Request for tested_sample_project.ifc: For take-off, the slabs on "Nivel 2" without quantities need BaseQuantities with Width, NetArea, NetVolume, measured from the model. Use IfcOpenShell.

First a look at what the model holds.

```python
import ifcopenshell
import ifcopenshell.util.element
import ifcopenshell.util.unit

model = ifcopenshell.open("tested_sample_project.ifc")
print(model.schema)
for unit_type in ("LENGTHUNIT", "AREAUNIT", "VOLUMEUNIT"):
    print(unit_type, ifcopenshell.util.unit.calculate_unit_scale(model, unit_type))
storey = next(s for s in model.by_type("IfcBuildingStorey") if s.Name == "Nivel 2")
slabs = [e for e in ifcopenshell.util.element.get_decomposition(storey) if e.is_a("IfcSlab")]
for e in sorted(slabs, key=lambda e: e.id()):
    print(e.id(), e.is_a(), e.Name, list(ifcopenshell.util.element.get_psets(e, qtos_only=True)), sep=" | ")
```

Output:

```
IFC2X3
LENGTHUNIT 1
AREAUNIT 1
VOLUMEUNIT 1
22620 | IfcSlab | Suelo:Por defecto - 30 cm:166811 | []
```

```python
import ifcopenshell
import ifcopenshell.api.pset
import ifcopenshell.geom
import ifcopenshell.util.element
import ifcopenshell.util.shape
import ifcopenshell.util.unit

model = ifcopenshell.open("tested_sample_project.ifc")
unit_scale = ifcopenshell.util.unit.calculate_unit_scale(model)
area_scale = ifcopenshell.util.unit.calculate_unit_scale(model, "AREAUNIT")
volume_scale = ifcopenshell.util.unit.calculate_unit_scale(model, "VOLUMEUNIT")
settings = ifcopenshell.geom.settings()

storey = next(s for s in model.by_type("IfcBuildingStorey") if s.Name == "Nivel 2")
slabs = [e for e in ifcopenshell.util.element.get_decomposition(storey) if e.is_a("IfcSlab")]

for e in sorted(slabs, key=lambda e: e.id()):
    if ifcopenshell.util.element.get_psets(e, qtos_only=True, should_inherit=False):
        continue
    # Geometry comes back in metres, in the element's own axes.
    shape = ifcopenshell.geom.create_shape(settings, e)
    values = {
        "Width": ifcopenshell.util.shape.get_z(shape.geometry) / unit_scale,
        "NetArea": ifcopenshell.util.shape.get_footprint_area(shape.geometry) / area_scale,
        "NetVolume": ifcopenshell.util.shape.get_volume(shape.geometry) / volume_scale,
    }
    qto = ifcopenshell.api.pset.add_qto(model, product=e, name="BaseQuantities")
    ifcopenshell.api.pset.edit_qto(model, qto=qto, properties=values)
    print(e.id(), {k: round(v, 3) for k, v in values.items()})

model.write("tested_sample_project-out.ifc")
```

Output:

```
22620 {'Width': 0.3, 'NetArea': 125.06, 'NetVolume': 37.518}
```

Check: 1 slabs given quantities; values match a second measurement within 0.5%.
